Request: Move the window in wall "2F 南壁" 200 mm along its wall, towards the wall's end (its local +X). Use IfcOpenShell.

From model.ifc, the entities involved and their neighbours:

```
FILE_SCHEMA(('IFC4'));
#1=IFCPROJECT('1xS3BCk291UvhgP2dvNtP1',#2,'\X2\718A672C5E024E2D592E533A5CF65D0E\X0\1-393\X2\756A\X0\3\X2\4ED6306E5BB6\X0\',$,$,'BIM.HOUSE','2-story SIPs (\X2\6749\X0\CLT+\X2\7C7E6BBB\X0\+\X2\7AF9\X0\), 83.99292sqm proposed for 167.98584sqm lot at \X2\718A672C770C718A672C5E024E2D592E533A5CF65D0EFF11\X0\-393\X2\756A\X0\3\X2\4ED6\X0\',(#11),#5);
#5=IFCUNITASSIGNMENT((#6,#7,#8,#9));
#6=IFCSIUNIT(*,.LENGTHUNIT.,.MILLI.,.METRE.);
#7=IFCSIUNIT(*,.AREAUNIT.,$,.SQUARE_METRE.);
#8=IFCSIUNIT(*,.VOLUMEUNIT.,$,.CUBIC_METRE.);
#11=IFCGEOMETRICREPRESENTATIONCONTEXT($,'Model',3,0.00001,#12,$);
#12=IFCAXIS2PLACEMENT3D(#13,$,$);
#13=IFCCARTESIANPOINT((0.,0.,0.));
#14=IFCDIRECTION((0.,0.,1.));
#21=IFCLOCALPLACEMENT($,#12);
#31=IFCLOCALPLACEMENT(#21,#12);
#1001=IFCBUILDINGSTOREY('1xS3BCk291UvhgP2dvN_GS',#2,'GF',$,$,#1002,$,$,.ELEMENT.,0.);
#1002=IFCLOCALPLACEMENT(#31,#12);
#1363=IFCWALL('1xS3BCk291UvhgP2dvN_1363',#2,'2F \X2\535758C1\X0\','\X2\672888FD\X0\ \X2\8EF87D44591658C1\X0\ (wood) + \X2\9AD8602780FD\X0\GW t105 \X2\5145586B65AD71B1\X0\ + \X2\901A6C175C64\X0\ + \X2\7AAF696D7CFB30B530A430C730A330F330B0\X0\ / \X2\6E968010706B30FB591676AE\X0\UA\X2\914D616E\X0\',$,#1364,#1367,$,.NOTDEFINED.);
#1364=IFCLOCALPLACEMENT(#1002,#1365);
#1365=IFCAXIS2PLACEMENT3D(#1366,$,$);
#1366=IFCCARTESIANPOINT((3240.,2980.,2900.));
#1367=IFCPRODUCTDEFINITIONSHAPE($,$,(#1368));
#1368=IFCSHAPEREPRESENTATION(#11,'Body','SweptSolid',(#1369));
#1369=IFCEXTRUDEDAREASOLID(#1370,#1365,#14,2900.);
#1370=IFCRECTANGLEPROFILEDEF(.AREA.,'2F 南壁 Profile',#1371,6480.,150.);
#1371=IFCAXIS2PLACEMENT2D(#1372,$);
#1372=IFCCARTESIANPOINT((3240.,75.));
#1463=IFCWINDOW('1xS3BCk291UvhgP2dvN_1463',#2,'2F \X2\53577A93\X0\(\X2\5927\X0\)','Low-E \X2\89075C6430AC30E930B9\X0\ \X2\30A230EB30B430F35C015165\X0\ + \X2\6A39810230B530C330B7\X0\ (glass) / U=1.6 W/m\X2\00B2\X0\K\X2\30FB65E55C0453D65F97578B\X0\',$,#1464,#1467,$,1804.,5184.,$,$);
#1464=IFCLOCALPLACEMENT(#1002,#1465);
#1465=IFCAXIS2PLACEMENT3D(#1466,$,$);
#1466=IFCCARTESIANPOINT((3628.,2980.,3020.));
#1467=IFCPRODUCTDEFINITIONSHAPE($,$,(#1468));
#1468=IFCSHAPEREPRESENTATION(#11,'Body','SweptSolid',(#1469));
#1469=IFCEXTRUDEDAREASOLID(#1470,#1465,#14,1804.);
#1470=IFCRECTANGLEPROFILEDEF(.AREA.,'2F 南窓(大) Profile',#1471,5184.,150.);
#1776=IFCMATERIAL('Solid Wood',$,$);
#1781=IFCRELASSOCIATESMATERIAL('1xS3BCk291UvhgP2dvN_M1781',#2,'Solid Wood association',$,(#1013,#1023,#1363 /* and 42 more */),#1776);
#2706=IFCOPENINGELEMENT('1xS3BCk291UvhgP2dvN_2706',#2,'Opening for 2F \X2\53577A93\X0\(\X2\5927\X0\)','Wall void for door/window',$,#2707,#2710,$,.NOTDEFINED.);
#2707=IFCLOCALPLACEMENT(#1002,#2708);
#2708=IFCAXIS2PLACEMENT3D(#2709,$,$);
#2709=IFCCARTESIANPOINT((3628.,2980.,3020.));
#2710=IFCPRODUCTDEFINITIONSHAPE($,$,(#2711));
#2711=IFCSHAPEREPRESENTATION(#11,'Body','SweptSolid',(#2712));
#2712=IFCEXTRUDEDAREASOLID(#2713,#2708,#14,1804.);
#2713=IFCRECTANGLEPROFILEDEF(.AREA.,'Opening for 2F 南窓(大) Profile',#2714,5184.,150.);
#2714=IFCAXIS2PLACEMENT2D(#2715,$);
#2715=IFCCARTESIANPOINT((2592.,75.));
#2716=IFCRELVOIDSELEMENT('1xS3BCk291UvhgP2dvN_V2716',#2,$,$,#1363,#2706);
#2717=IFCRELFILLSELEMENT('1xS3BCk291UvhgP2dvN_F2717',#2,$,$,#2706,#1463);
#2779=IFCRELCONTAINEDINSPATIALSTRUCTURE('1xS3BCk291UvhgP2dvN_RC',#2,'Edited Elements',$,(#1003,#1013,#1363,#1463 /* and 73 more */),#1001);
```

```python
import ifcopenshell
import ifcopenshell.api.geometry
import ifcopenshell.util.placement
import ifcopenshell.util.unit

model = ifcopenshell.open("model.ifc")
unit_scale = ifcopenshell.util.unit.calculate_unit_scale(model)

window = model.by_guid("1xS3BCk291UvhgP2dvN_1463")
opening = window.FillsVoids[0].RelatingOpeningElement
wall = opening.VoidsElements[0].RelatingBuildingElement

wall_matrix = ifcopenshell.util.placement.get_local_placement(wall.ObjectPlacement)
shift = wall_matrix[:3, 0] * 0.2 / unit_scale
before = ifcopenshell.util.placement.get_local_placement(window.ObjectPlacement)[:3, 3].copy()

# The window is not placed relative to its opening, so move both.
for product in (opening, window):
    matrix = ifcopenshell.util.placement.get_local_placement(product.ObjectPlacement)
    matrix[:3, 3] += shift
    ifcopenshell.api.geometry.edit_object_placement(model, product=product, matrix=matrix, is_si=False)

after = ifcopenshell.util.placement.get_local_placement(window.ObjectPlacement)[:3, 3]
print("window moved by", (after - before).round(3) + 0.0)

model.write("model_updated.ifc")
```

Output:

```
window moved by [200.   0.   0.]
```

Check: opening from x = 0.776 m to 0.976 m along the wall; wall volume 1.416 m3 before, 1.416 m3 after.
